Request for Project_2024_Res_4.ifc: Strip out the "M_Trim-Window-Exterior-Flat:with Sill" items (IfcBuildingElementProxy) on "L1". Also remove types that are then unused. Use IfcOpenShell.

First a look at what the model holds.

```python
import ifcopenshell
import ifcopenshell.util.element

model = ifcopenshell.open("Project_2024_Res_4.ifc")
print(model.schema)
storey = next(s for s in model.by_type("IfcBuildingStorey") if s.Name == "L1")
proxies = [e for e in ifcopenshell.util.element.get_decomposition(storey) if e.is_a("IfcBuildingElementProxy")]
seen = {}
for e in proxies:
    element_type = ifcopenshell.util.element.get_type(e)
    name = element_type.Name if element_type not in (None, e) else None
    seen[name] = seen.get(name, 0) + 1
for name, count in sorted(seen.items(), key=str):
    print(count, "x", name)
```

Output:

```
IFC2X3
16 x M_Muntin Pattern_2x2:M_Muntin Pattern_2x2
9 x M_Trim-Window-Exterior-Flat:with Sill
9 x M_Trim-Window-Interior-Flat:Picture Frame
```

```python
import ifcopenshell
import ifcopenshell.api.root
import ifcopenshell.util.element

model = ifcopenshell.open("Project_2024_Res_4.ifc")

storey = next(s for s in model.by_type("IfcBuildingStorey") if s.Name == "L1")
proxies = [e for e in ifcopenshell.util.element.get_decomposition(storey) if e.is_a("IfcBuildingElementProxy")]
targets = [e for e in proxies if (t := ifcopenshell.util.element.get_type(e)) not in (None, e) and t.Name == "M_Trim-Window-Exterior-Flat:with Sill"]
types = {ifcopenshell.util.element.get_type(e) for e in targets} - {None, *targets}

for e in targets:
    ifcopenshell.api.root.remove_product(model, product=e)
print(len(targets), "removed")

unused = [t for t in types if not ifcopenshell.util.element.get_types(t)]
for t in unused:
    ifcopenshell.api.root.remove_product(model, product=t)
print(len(unused), "unused types removed")

model.write("Project_2024_Res_4-out.ifc")
```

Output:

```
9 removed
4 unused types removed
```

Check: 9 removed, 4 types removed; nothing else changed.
